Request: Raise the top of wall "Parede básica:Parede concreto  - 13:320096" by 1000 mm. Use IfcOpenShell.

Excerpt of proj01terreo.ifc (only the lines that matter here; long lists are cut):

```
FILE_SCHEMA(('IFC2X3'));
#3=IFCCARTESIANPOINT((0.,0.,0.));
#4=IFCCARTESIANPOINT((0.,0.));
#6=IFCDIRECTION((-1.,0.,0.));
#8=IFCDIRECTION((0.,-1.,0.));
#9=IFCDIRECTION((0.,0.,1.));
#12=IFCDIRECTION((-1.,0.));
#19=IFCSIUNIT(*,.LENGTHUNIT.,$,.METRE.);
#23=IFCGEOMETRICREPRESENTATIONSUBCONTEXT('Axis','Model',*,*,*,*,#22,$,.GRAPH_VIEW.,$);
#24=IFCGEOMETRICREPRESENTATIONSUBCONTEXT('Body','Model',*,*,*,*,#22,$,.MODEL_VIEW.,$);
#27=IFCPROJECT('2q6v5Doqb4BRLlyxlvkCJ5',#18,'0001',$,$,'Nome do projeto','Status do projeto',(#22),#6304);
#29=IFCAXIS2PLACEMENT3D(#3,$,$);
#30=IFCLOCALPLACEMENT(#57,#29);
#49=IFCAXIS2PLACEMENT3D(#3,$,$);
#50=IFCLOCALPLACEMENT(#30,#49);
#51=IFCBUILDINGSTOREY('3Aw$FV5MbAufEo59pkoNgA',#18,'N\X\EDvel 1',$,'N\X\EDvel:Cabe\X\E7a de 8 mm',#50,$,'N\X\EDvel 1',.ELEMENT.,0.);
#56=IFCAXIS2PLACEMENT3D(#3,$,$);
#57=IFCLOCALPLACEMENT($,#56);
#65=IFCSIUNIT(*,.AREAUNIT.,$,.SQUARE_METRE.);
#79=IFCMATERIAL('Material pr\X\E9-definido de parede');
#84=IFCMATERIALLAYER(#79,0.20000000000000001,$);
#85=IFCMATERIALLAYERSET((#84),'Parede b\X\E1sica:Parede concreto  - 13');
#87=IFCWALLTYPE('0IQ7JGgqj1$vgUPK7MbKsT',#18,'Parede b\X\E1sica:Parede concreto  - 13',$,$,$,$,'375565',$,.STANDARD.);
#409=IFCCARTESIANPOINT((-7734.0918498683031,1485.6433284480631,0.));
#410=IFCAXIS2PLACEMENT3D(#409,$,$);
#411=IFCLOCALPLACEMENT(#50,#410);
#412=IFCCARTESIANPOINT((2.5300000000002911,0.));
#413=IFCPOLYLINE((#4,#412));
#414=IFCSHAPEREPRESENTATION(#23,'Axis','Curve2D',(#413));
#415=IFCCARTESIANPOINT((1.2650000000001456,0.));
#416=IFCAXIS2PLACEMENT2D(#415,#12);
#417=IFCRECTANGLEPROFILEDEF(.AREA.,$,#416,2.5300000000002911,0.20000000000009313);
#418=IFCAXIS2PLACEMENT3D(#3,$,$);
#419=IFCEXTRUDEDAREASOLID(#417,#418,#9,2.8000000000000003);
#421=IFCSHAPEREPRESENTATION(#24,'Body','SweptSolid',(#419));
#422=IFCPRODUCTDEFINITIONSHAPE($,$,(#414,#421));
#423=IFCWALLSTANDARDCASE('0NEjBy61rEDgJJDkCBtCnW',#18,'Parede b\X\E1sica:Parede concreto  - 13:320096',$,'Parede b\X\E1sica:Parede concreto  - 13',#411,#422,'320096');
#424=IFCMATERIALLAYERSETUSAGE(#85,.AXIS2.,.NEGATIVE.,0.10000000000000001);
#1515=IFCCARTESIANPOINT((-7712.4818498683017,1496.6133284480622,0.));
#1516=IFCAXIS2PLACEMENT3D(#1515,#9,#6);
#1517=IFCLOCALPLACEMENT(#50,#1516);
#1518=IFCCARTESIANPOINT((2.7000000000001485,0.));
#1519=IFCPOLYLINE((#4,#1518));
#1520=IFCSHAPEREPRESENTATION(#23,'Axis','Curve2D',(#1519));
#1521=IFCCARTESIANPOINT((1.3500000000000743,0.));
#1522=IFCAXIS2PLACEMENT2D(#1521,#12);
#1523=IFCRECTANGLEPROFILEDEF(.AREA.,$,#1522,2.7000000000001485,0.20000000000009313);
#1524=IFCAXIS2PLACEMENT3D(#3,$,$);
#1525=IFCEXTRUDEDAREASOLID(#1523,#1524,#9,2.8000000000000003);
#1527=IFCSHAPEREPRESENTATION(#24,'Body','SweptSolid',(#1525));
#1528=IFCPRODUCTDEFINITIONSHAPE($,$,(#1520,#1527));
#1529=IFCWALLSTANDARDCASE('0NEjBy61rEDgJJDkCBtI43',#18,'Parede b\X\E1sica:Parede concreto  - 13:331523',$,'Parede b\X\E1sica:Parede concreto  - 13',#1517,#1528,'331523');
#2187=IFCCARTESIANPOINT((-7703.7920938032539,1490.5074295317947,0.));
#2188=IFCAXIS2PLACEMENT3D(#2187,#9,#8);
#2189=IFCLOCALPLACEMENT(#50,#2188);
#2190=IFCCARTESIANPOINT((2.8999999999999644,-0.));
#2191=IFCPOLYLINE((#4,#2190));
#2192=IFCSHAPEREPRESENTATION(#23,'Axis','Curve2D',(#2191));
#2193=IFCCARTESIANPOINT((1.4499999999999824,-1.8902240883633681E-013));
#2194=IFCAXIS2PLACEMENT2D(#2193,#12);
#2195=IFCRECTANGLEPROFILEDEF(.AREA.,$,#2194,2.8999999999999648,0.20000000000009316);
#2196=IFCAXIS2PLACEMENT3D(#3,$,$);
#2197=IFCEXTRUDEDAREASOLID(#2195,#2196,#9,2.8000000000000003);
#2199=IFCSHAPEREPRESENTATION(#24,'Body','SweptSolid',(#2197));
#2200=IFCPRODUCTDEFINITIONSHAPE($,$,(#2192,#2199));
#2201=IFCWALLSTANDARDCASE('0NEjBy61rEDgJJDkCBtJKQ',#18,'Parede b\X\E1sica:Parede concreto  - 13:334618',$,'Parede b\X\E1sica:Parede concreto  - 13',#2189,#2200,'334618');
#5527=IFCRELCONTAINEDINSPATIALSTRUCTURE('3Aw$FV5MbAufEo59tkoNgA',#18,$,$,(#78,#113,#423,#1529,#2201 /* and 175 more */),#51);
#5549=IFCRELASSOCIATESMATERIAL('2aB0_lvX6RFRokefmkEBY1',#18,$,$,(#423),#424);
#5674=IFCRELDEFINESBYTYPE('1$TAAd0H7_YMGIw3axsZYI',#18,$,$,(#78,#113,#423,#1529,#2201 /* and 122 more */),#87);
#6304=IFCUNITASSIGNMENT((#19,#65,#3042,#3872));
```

```python
import ifcopenshell
import ifcopenshell.geom
import ifcopenshell.util.representation
import ifcopenshell.util.shape
import ifcopenshell.util.unit

model = ifcopenshell.open("proj01terreo.ifc")
unit_scale = ifcopenshell.util.unit.calculate_unit_scale(model)
settings = ifcopenshell.geom.settings()


def volume(element):
    """Net volume in cubic metres, openings subtracted."""
    shape = ifcopenshell.geom.create_shape(settings, element)
    return ifcopenshell.util.shape.get_volume(shape.geometry)


wall = model.by_guid("0NEjBy61rEDgJJDkCBtCnW")
before = volume(wall)

body = ifcopenshell.util.representation.get_representation(wall, "Model", "Body")
solid = body.Items[0]
old_height = solid.Depth
solid.Depth += 1 / unit_scale
after = volume(wall)

print(f"height {old_height:g} -> {solid.Depth:g}, volume {before:.3f} -> {after:.3f} m3")

model.write("proj01terreo_updated.ifc")
```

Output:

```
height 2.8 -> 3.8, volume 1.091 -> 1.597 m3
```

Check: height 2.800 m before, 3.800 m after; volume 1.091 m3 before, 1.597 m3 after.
